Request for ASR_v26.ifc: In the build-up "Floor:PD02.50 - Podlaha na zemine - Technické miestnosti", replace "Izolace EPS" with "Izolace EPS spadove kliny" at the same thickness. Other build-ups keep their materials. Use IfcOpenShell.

First a look at what the model holds.

```python
import ifcopenshell
import ifcopenshell.util.element

model = ifcopenshell.open("ASR_v26.ifc")
print(model.schema)
for layer_set in model.by_type("IfcMaterialLayerSet"):
    if layer_set.LayerSetName == "Floor:PD02.50 - Podlaha na zemine - Technické miestnosti":
        for layer in layer_set.MaterialLayers:
            print(layer.id(), layer.Material and layer.Material.Name, layer.LayerThickness, sep=" | ")
        print(len(ifcopenshell.util.element.get_elements_by_material(model, layer_set)), "elements and types use it")
print(sorted(m.Name for m in model.by_type("IfcMaterial") if m.Name)[:60])
```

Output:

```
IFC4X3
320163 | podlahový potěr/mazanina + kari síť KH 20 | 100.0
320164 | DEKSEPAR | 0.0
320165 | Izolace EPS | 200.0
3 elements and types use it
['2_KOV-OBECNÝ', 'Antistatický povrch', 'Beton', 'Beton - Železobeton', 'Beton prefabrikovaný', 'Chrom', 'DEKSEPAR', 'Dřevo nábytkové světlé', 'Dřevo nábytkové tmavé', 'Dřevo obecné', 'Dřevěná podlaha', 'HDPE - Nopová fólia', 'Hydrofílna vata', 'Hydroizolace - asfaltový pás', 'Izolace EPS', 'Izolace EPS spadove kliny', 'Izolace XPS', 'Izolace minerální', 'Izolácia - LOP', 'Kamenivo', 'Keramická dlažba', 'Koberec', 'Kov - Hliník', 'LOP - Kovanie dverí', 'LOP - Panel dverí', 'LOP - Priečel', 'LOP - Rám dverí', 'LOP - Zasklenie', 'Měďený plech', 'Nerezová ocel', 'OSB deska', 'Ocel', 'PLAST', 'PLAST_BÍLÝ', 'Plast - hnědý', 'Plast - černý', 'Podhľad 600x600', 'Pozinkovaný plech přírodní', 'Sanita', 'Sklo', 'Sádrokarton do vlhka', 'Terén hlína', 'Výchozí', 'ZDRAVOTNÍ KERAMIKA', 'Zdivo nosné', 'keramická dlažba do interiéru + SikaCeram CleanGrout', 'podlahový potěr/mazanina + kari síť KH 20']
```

```python
import ifcopenshell
import ifcopenshell.api.material

model = ifcopenshell.open("ASR_v26.ifc")

layer_set = next(s for s in model.by_type("IfcMaterialLayerSet") if s.LayerSetName == "Floor:PD02.50 - Podlaha na zemine - Technické miestnosti")
layer = next(l for l in layer_set.MaterialLayers if l.Material and l.Material.Name == "Izolace EPS")
material = next(m for m in model.by_type("IfcMaterial") if m.Name == "Izolace EPS spadove kliny")

# Point this one layer at the other material; renaming the old one would change it everywhere.
ifcopenshell.api.material.edit_layer(model, layer=layer, attributes={"Name": material.Name}, material=material)

print([l.Material.Name if l.Material else None for l in layer_set.MaterialLayers])

model.write("ASR_v26_edited.ifc")
```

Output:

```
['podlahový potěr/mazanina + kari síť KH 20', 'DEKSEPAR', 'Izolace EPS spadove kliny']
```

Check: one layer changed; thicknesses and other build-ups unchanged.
